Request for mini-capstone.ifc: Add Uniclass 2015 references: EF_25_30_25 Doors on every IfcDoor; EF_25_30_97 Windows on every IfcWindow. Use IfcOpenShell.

First a look at what the model holds.

```python
import ifcopenshell

model = ifcopenshell.open("mini-capstone.ifc")
print(model.schema)
print("classifications:", [c.Name for c in model.by_type("IfcClassification")])
for ifc_class in ("IfcDoor", "IfcRoof", "IfcStair", "IfcWall", "IfcWindow"):
    print(ifc_class, len(model.by_type(ifc_class)))
```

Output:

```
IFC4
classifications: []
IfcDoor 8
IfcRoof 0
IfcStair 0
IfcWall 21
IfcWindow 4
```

```python
import ifcopenshell
import ifcopenshell.api.classification

model = ifcopenshell.open("mini-capstone.ifc")

system = ifcopenshell.api.classification.add_classification(model, classification="Uniclass 2015")

codes = {
    "IfcDoor": ("EF_25_30_25", "Doors"),
    "IfcWindow": ("EF_25_30_97", "Windows"),
}
for ifc_class, (code, name) in codes.items():
    products = model.by_type(ifc_class)
    ifcopenshell.api.classification.add_reference(
        model, products=products, classification=system, identification=code, name=name
    )
    print(code, len(products))

model.write("mini-capstone_v2.ifc")
```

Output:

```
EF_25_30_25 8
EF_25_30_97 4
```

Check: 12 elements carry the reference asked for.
